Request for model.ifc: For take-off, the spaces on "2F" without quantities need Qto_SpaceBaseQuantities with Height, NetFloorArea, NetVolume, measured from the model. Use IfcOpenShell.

First a look at what the model holds.

```python
import ifcopenshell
import ifcopenshell.util.element
import ifcopenshell.util.unit

model = ifcopenshell.open("model.ifc")
print(model.schema)
for unit_type in ("LENGTHUNIT", "AREAUNIT", "VOLUMEUNIT"):
    print(unit_type, ifcopenshell.util.unit.calculate_unit_scale(model, unit_type))
storey = next(s for s in model.by_type("IfcBuildingStorey") if s.Name == "2F")
spaces = [e for e in ifcopenshell.util.element.get_decomposition(storey) if e.is_a("IfcSpace")]
for e in sorted(spaces, key=lambda e: e.id()):
    print(e.id(), e.is_a(), e.Name, list(ifcopenshell.util.element.get_psets(e, qtos_only=True)), sep=" | ")
```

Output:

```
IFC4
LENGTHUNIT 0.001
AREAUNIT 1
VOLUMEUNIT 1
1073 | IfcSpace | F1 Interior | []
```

```python
import ifcopenshell
import ifcopenshell.api.pset
import ifcopenshell.geom
import ifcopenshell.util.element
import ifcopenshell.util.shape
import ifcopenshell.util.unit

model = ifcopenshell.open("model.ifc")
unit_scale = ifcopenshell.util.unit.calculate_unit_scale(model)
area_scale = ifcopenshell.util.unit.calculate_unit_scale(model, "AREAUNIT")
volume_scale = ifcopenshell.util.unit.calculate_unit_scale(model, "VOLUMEUNIT")
settings = ifcopenshell.geom.settings()

storey = next(s for s in model.by_type("IfcBuildingStorey") if s.Name == "2F")
spaces = [e for e in ifcopenshell.util.element.get_decomposition(storey) if e.is_a("IfcSpace")]

for e in sorted(spaces, key=lambda e: e.id()):
    if ifcopenshell.util.element.get_psets(e, qtos_only=True, should_inherit=False):
        continue
    # Geometry comes back in metres, in the element's own axes.
    shape = ifcopenshell.geom.create_shape(settings, e)
    values = {
        "Height": ifcopenshell.util.shape.get_z(shape.geometry) / unit_scale,
        "NetFloorArea": ifcopenshell.util.shape.get_footprint_area(shape.geometry) / area_scale,
        "NetVolume": ifcopenshell.util.shape.get_volume(shape.geometry) / volume_scale,
    }
    qto = ifcopenshell.api.pset.add_qto(model, product=e, name="Qto_SpaceBaseQuantities")
    ifcopenshell.api.pset.edit_qto(model, qto=qto, properties=values)
    print(e.id(), {k: round(v, 3) for k, v in values.items()})

model.write("model_rev.ifc")
```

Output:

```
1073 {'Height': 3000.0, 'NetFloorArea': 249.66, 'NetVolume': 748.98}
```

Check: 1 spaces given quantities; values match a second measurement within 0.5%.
